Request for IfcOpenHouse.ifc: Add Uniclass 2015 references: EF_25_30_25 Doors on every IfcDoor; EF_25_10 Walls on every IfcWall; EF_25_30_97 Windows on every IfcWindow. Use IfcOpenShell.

First a look at what the model holds.

```python
import ifcopenshell

model = ifcopenshell.open("IfcOpenHouse.ifc")
print(model.schema)
print("classifications:", [c.Name for c in model.by_type("IfcClassification")])
for ifc_class in ("IfcDoor", "IfcRoof", "IfcStair", "IfcWall", "IfcWindow"):
    print(ifc_class, len(model.by_type(ifc_class)))
```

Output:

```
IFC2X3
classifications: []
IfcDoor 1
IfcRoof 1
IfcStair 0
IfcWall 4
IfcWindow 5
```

```python
import ifcopenshell
import ifcopenshell.api.classification

model = ifcopenshell.open("IfcOpenHouse.ifc")

# IFC2X3 requires Source and Edition and has no link from the project to the system.
system = model.create_entity("IfcClassification", Source="NBS", Edition="2015", Name="Uniclass 2015")

codes = {
    "IfcDoor": ("EF_25_30_25", "Doors"),
    "IfcWall": ("EF_25_10", "Walls"),
    "IfcWindow": ("EF_25_30_97", "Windows"),
}
for ifc_class, (code, name) in codes.items():
    products = model.by_type(ifc_class)
    ifcopenshell.api.classification.add_reference(
        model, products=products, classification=system, identification=code, name=name
    )
    print(code, len(products))

model.write("IfcOpenHouse_v2.ifc")
```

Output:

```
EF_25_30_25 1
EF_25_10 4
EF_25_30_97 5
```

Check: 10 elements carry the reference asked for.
